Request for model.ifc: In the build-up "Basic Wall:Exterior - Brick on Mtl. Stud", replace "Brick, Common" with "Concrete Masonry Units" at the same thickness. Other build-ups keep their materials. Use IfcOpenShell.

First a look at what the model holds.

```python
import ifcopenshell
import ifcopenshell.util.element

model = ifcopenshell.open("model.ifc")
print(model.schema)
for layer_set in model.by_type("IfcMaterialLayerSet"):
    if layer_set.LayerSetName == "Basic Wall:Exterior - Brick on Mtl. Stud":
        for layer in layer_set.MaterialLayers:
            print(layer.id(), layer.Material and layer.Material.Name, layer.LayerThickness, sep=" | ")
        print(len(ifcopenshell.util.element.get_elements_by_material(model, layer_set)), "elements and types use it")
print(sorted(m.Name for m in model.by_type("IfcMaterial") if m.Name)[:60])
```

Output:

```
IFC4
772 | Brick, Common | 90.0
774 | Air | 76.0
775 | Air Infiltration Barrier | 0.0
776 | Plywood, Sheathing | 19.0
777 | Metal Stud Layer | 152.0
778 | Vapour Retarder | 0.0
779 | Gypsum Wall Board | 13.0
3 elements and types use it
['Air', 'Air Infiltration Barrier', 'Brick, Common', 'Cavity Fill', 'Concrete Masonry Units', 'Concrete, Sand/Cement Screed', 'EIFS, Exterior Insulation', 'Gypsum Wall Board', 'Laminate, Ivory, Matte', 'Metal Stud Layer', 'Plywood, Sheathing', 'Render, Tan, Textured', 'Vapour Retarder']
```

```python
import ifcopenshell
import ifcopenshell.api.material

model = ifcopenshell.open("model.ifc")

layer_set = next(s for s in model.by_type("IfcMaterialLayerSet") if s.LayerSetName == "Basic Wall:Exterior - Brick on Mtl. Stud")
layer = next(l for l in layer_set.MaterialLayers if l.Material and l.Material.Name == "Brick, Common")
material = next(m for m in model.by_type("IfcMaterial") if m.Name == "Concrete Masonry Units")

# Point this one layer at the other material; renaming the old one would change it everywhere.
ifcopenshell.api.material.edit_layer(model, layer=layer, attributes={}, material=material)

print([l.Material.Name if l.Material else None for l in layer_set.MaterialLayers])

model.write("model_v2.ifc")
```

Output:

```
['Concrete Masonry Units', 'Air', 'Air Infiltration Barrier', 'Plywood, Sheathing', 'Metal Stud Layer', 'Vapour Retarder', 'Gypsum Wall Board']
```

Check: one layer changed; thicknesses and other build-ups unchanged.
